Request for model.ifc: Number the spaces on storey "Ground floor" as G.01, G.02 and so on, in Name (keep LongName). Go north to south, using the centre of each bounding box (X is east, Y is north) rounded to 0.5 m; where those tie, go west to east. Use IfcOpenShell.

First a look at what the model holds.

```python
import ifcopenshell
import ifcopenshell.util.element
import ifcopenshell.util.placement

model = ifcopenshell.open("model.ifc")
print(model.schema)
storey = next(s for s in model.by_type("IfcBuildingStorey") if s.Name == "Ground floor")
spaces = [e for e in ifcopenshell.util.element.get_decomposition(storey) if e.is_a("IfcSpace")]
for e in sorted(spaces, key=lambda e: e.id()):
    origin = ifcopenshell.util.placement.get_local_placement(e.ObjectPlacement)[:3, 3]
    print(e.id(), e.Name, e.LongName, origin.round(2) + 0.0, sep=" | ")
```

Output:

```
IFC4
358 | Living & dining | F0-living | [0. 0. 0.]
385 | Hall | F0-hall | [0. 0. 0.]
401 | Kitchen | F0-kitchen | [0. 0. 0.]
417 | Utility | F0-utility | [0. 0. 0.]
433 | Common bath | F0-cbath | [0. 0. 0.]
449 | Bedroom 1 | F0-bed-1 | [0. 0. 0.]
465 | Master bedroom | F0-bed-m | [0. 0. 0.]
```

```python
import ifcopenshell
import ifcopenshell.geom
import ifcopenshell.util.element
import ifcopenshell.util.shape

model = ifcopenshell.open("model.ifc")
settings = ifcopenshell.geom.settings()
settings.set("use-world-coords", True)


def centre(element):
    shape = ifcopenshell.geom.create_shape(settings, element)
    return ifcopenshell.util.shape.get_bbox_centroid(shape.geometry)


storey = next(s for s in model.by_type("IfcBuildingStorey") if s.Name == "Ground floor")
spaces = [e for e in ifcopenshell.util.element.get_decomposition(storey) if e.is_a("IfcSpace")]

# Insertion points can sit at a corner or the storey origin, so sort by the geometry (in metres).
centres = {e: centre(e) for e in spaces}
spaces.sort(key=lambda e: (-round(centres[e][1] / 0.5), centres[e][0]))

for i, e in enumerate(spaces, start=1):
    number = f"G.{i:02d}"
    e.Name = number
    print(e.id(), number)

model.write("model_edited.ifc")
```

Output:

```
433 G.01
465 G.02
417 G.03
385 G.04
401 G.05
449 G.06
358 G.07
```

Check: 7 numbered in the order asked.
